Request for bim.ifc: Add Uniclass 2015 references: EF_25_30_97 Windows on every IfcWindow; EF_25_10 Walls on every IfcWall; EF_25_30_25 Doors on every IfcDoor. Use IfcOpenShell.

First a look at what the model holds.

```python
import ifcopenshell

model = ifcopenshell.open("bim.ifc")
print(model.schema)
print("classifications:", [c.Name for c in model.by_type("IfcClassification")])
for ifc_class in ("IfcDoor", "IfcRoof", "IfcStair", "IfcWall", "IfcWindow"):
    print(ifc_class, len(model.by_type(ifc_class)))
```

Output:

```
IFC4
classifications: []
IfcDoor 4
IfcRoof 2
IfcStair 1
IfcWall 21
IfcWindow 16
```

```python
import ifcopenshell
import ifcopenshell.api.classification

model = ifcopenshell.open("bim.ifc")

system = ifcopenshell.api.classification.add_classification(model, classification="Uniclass 2015")

codes = {
    "IfcWindow": ("EF_25_30_97", "Windows"),
    "IfcWall": ("EF_25_10", "Walls"),
    "IfcDoor": ("EF_25_30_25", "Doors"),
}
for ifc_class, (code, name) in codes.items():
    products = model.by_type(ifc_class)
    ifcopenshell.api.classification.add_reference(
        model, products=products, classification=system, identification=code, name=name
    )
    print(code, len(products))

model.write("bim-out.ifc")
```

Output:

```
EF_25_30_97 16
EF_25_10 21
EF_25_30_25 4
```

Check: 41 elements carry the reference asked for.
